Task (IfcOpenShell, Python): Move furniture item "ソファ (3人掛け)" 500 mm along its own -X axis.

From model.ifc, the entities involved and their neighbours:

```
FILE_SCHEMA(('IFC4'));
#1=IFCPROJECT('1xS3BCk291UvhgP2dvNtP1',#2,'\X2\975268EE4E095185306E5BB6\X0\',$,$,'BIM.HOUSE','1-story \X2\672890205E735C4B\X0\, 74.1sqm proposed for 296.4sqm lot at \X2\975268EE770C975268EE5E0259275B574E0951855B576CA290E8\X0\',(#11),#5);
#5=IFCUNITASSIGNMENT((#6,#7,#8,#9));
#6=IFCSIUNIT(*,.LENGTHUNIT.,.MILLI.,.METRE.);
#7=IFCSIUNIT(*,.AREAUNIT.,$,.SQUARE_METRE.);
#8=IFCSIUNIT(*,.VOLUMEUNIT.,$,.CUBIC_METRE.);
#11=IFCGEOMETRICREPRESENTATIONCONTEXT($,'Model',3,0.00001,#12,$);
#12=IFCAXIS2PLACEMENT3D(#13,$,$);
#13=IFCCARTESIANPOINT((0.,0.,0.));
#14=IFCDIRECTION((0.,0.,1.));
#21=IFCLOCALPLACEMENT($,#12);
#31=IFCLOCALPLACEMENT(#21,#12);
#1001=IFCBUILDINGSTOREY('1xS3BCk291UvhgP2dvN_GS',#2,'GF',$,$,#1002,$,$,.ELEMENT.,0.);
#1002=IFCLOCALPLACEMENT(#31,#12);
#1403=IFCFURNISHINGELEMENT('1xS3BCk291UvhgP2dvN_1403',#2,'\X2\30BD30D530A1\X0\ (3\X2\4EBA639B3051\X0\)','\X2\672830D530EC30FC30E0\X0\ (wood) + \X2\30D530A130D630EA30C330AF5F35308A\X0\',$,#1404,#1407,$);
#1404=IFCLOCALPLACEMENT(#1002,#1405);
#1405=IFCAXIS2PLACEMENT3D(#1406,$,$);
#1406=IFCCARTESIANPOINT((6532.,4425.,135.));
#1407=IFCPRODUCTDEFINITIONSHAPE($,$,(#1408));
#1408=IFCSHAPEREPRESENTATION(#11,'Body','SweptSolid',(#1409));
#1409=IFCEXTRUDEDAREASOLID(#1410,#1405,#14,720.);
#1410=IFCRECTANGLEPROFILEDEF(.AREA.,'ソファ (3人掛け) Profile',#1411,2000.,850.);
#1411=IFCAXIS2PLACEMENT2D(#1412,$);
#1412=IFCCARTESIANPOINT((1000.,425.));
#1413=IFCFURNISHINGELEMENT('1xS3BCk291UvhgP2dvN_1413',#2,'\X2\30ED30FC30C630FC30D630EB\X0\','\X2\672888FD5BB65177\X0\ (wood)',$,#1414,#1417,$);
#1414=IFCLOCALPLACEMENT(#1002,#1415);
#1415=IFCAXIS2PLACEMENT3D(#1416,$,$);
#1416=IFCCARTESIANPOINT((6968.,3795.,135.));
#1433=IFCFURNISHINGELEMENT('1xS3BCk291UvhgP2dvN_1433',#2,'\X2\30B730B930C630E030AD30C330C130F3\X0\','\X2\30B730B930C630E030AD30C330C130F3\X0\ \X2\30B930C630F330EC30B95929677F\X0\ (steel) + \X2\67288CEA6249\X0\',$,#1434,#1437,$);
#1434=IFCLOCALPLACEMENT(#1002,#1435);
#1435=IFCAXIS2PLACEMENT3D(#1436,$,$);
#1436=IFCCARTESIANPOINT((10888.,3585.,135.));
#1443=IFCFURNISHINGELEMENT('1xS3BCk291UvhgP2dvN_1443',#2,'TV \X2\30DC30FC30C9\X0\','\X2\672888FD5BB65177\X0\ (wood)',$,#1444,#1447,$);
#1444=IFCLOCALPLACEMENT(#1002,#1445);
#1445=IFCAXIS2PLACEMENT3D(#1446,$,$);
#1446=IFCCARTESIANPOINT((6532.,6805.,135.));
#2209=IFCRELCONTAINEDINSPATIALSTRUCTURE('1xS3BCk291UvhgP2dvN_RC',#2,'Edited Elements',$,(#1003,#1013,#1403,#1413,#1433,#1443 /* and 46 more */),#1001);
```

```python
import ifcopenshell
import ifcopenshell.api.geometry
import ifcopenshell.util.placement
import ifcopenshell.util.unit

model = ifcopenshell.open("model.ifc")
unit_scale = ifcopenshell.util.unit.calculate_unit_scale(model)

item = model.by_guid("1xS3BCk291UvhgP2dvN_1403")
matrix = ifcopenshell.util.placement.get_local_placement(item.ObjectPlacement)
matrix[:3, 3] -= matrix[:3, 0] * 0.5 / unit_scale
ifcopenshell.api.geometry.edit_object_placement(model, product=item, matrix=matrix, is_si=False)

print(ifcopenshell.util.placement.get_local_placement(item.ObjectPlacement).round(3) + 0.0)

model.write("model_v2.ifc")
```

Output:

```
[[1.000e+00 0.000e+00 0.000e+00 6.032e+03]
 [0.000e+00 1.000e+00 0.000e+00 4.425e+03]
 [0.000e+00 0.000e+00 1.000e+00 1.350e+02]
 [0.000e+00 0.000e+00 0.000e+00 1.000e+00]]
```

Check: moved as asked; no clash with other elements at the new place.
